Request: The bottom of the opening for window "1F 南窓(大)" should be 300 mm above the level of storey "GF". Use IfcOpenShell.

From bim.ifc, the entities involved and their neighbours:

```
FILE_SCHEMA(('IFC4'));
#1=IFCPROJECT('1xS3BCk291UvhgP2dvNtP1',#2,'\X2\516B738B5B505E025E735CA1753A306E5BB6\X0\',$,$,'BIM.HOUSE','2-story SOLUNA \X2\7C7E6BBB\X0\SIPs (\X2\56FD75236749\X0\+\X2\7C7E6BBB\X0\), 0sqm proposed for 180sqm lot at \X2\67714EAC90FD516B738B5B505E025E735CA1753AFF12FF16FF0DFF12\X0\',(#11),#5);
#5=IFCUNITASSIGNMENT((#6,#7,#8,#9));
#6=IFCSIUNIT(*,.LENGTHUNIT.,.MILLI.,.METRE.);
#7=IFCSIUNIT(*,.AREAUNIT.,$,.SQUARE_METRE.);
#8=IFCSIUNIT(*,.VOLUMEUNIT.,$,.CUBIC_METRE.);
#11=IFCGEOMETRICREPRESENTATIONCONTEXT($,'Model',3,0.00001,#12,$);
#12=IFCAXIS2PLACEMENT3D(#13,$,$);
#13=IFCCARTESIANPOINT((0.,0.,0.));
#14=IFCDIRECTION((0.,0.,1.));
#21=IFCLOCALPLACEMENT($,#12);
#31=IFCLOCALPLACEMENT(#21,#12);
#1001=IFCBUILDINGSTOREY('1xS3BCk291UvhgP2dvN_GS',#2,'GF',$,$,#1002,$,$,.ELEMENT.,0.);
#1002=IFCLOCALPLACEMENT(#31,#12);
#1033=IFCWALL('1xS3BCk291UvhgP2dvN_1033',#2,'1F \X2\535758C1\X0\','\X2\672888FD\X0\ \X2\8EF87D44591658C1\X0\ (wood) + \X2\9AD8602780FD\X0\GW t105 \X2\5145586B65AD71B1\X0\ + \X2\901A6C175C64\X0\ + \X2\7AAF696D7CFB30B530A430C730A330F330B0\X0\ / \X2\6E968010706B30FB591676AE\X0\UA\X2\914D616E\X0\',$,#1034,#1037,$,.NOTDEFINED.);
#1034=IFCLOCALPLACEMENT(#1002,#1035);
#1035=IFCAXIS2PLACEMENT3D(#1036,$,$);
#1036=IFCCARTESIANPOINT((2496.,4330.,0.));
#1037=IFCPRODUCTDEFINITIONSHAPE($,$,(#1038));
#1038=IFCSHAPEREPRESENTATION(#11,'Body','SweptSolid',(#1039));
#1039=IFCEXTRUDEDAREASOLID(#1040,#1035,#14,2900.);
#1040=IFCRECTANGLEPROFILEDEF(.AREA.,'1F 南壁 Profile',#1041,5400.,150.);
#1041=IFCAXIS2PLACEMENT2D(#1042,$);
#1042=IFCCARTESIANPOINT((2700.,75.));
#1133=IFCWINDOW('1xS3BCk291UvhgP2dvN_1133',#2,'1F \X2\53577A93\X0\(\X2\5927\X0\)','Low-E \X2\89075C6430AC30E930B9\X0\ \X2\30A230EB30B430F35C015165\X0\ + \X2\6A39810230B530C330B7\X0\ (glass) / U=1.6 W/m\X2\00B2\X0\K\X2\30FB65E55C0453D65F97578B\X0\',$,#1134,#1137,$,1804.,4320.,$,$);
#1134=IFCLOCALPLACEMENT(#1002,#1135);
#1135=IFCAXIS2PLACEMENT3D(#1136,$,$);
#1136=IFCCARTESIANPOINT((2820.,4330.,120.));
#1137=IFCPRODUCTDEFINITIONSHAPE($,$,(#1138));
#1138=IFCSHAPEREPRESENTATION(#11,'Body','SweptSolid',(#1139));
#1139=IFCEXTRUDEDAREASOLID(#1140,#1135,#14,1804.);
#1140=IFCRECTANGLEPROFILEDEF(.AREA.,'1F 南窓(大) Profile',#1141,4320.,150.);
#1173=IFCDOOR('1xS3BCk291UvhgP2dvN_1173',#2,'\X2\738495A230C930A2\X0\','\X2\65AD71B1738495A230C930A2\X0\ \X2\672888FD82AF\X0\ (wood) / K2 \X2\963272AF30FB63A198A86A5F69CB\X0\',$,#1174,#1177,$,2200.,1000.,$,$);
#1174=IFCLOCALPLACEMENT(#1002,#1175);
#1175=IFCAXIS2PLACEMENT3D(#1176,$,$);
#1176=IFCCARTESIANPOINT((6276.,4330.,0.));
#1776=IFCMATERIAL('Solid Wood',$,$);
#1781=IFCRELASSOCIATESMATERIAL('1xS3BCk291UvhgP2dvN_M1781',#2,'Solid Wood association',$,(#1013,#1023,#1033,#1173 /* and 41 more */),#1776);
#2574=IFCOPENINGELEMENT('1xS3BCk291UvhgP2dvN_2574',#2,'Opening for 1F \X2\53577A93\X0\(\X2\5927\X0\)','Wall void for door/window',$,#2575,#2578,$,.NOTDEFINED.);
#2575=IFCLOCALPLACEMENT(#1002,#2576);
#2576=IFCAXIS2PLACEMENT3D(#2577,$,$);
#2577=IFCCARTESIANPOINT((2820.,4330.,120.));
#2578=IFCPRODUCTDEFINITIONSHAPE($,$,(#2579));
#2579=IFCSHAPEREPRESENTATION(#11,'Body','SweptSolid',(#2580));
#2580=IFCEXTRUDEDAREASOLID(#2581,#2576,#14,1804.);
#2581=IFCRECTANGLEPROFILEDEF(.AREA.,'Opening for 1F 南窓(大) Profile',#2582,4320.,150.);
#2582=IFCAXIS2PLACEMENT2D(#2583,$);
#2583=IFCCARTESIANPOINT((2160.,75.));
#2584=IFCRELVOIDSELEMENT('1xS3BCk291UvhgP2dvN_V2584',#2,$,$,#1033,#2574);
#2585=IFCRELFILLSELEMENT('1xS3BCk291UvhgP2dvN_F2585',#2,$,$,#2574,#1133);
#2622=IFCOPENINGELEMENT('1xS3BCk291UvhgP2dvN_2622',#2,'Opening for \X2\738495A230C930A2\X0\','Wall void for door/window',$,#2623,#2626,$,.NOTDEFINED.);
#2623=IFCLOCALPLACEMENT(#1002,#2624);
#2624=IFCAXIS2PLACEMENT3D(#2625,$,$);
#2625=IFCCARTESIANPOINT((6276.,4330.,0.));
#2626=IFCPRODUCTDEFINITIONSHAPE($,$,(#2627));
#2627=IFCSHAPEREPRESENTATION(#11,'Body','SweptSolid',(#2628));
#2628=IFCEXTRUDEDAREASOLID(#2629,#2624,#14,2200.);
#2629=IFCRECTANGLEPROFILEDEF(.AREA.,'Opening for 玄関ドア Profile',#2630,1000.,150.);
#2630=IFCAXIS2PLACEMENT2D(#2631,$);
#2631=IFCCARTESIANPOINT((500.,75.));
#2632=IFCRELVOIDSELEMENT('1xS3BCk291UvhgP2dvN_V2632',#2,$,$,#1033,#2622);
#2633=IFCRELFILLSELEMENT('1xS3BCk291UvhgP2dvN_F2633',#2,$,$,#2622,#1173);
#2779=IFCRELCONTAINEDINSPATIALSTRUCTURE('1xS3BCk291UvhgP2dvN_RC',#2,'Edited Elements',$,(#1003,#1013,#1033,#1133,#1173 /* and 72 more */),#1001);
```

```python
import numpy as np
import ifcopenshell
import ifcopenshell.api.geometry
import ifcopenshell.geom
import ifcopenshell.util.element
import ifcopenshell.util.placement
import ifcopenshell.util.shape
import ifcopenshell.util.unit

model = ifcopenshell.open("bim.ifc")
unit_scale = ifcopenshell.util.unit.calculate_unit_scale(model)

window = model.by_id(1133)
opening = window.FillsVoids[0].RelatingOpeningElement
storey = ifcopenshell.util.element.get_container(window, ifc_class="IfcBuildingStorey")
level = ifcopenshell.util.placement.get_local_placement(storey.ObjectPlacement)[2, 3]

# The opening's origin need not be at the sill, so measure its lowest point.
shape = ifcopenshell.geom.create_shape(ifcopenshell.geom.settings(), opening)
bottom = ifcopenshell.util.shape.get_shape_bottom_elevation(shape, shape.geometry) / unit_scale
dz = level + 0.3 / unit_scale - bottom

shift = np.array([0.0, 0.0, dz])
# The window is not placed relative to its opening, so move both.
for product in (opening, window):
    matrix = ifcopenshell.util.placement.get_local_placement(product.ObjectPlacement)
    matrix[:3, 3] += shift
    ifcopenshell.api.geometry.edit_object_placement(model, product=product, matrix=matrix, is_si=False)

print(f"moved by {dz * unit_scale:+.3f} m")

model.write("bim_updated.ifc")
```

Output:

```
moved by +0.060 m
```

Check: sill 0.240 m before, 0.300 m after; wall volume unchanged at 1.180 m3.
